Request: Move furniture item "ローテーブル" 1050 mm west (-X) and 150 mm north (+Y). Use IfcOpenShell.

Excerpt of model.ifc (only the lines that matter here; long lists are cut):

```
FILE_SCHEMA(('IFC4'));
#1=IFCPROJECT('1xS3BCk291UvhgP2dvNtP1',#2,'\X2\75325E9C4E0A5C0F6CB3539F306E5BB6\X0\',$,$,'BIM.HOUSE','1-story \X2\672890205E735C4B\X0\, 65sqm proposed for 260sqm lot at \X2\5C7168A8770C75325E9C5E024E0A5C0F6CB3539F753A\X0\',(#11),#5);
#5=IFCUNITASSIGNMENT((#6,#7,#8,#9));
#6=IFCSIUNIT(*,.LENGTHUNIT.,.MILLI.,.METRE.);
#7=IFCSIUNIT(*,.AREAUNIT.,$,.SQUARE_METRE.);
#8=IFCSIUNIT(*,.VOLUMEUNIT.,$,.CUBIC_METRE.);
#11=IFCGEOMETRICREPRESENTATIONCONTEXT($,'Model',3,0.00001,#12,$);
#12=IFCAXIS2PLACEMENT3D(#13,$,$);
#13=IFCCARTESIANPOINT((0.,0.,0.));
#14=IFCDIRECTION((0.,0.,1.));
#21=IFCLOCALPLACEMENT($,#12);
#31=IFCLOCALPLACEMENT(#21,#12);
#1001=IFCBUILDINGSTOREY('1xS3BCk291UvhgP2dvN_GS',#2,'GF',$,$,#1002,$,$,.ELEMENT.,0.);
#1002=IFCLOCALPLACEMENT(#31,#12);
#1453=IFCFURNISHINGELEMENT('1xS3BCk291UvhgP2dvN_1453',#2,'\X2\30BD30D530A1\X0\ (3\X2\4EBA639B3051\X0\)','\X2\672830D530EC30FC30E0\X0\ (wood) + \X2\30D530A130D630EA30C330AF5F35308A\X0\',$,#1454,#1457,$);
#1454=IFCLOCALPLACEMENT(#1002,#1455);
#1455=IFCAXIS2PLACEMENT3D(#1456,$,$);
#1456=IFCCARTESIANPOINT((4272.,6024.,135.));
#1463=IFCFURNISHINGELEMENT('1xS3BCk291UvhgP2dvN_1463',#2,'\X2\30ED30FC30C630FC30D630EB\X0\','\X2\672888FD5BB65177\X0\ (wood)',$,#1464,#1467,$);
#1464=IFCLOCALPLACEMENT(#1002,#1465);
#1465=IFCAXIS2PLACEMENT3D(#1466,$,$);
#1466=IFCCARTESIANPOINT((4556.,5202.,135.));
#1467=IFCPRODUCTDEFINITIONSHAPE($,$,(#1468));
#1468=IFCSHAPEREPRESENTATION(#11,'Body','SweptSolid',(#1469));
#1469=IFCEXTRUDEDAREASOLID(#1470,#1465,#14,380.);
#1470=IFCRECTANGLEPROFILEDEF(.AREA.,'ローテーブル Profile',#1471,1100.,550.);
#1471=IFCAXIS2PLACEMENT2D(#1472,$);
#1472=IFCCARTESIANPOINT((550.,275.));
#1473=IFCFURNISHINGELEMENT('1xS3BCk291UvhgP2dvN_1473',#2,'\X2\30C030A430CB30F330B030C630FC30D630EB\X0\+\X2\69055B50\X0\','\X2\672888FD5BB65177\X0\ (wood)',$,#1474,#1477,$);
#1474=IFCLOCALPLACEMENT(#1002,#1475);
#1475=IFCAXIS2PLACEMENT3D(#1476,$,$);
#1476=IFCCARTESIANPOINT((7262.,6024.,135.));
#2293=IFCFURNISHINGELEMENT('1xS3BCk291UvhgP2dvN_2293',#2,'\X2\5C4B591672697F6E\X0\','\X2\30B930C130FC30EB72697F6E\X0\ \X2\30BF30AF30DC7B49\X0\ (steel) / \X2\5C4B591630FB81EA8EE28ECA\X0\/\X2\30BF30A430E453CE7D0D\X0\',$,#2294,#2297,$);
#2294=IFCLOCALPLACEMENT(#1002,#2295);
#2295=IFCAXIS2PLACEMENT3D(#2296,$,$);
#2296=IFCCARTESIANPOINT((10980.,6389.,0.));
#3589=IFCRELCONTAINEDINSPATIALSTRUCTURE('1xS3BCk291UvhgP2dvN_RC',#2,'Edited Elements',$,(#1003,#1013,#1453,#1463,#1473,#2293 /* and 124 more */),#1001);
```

```python
import ifcopenshell
import ifcopenshell.api.geometry
import ifcopenshell.util.placement

model = ifcopenshell.open("model.ifc")

item = model.by_guid("1xS3BCk291UvhgP2dvN_1463")
matrix = ifcopenshell.util.placement.get_local_placement(item.ObjectPlacement)
matrix[0, 3] -= 1050.0
matrix[1, 3] += 150.0
ifcopenshell.api.geometry.edit_object_placement(model, product=item, matrix=matrix, is_si=False)

print(ifcopenshell.util.placement.get_local_placement(item.ObjectPlacement).round(3) + 0.0)

model.write("model_rev.ifc")
```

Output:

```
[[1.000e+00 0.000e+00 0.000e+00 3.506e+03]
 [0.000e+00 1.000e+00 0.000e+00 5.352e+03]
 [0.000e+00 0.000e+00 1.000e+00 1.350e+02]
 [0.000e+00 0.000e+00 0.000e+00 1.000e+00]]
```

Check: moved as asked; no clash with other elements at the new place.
